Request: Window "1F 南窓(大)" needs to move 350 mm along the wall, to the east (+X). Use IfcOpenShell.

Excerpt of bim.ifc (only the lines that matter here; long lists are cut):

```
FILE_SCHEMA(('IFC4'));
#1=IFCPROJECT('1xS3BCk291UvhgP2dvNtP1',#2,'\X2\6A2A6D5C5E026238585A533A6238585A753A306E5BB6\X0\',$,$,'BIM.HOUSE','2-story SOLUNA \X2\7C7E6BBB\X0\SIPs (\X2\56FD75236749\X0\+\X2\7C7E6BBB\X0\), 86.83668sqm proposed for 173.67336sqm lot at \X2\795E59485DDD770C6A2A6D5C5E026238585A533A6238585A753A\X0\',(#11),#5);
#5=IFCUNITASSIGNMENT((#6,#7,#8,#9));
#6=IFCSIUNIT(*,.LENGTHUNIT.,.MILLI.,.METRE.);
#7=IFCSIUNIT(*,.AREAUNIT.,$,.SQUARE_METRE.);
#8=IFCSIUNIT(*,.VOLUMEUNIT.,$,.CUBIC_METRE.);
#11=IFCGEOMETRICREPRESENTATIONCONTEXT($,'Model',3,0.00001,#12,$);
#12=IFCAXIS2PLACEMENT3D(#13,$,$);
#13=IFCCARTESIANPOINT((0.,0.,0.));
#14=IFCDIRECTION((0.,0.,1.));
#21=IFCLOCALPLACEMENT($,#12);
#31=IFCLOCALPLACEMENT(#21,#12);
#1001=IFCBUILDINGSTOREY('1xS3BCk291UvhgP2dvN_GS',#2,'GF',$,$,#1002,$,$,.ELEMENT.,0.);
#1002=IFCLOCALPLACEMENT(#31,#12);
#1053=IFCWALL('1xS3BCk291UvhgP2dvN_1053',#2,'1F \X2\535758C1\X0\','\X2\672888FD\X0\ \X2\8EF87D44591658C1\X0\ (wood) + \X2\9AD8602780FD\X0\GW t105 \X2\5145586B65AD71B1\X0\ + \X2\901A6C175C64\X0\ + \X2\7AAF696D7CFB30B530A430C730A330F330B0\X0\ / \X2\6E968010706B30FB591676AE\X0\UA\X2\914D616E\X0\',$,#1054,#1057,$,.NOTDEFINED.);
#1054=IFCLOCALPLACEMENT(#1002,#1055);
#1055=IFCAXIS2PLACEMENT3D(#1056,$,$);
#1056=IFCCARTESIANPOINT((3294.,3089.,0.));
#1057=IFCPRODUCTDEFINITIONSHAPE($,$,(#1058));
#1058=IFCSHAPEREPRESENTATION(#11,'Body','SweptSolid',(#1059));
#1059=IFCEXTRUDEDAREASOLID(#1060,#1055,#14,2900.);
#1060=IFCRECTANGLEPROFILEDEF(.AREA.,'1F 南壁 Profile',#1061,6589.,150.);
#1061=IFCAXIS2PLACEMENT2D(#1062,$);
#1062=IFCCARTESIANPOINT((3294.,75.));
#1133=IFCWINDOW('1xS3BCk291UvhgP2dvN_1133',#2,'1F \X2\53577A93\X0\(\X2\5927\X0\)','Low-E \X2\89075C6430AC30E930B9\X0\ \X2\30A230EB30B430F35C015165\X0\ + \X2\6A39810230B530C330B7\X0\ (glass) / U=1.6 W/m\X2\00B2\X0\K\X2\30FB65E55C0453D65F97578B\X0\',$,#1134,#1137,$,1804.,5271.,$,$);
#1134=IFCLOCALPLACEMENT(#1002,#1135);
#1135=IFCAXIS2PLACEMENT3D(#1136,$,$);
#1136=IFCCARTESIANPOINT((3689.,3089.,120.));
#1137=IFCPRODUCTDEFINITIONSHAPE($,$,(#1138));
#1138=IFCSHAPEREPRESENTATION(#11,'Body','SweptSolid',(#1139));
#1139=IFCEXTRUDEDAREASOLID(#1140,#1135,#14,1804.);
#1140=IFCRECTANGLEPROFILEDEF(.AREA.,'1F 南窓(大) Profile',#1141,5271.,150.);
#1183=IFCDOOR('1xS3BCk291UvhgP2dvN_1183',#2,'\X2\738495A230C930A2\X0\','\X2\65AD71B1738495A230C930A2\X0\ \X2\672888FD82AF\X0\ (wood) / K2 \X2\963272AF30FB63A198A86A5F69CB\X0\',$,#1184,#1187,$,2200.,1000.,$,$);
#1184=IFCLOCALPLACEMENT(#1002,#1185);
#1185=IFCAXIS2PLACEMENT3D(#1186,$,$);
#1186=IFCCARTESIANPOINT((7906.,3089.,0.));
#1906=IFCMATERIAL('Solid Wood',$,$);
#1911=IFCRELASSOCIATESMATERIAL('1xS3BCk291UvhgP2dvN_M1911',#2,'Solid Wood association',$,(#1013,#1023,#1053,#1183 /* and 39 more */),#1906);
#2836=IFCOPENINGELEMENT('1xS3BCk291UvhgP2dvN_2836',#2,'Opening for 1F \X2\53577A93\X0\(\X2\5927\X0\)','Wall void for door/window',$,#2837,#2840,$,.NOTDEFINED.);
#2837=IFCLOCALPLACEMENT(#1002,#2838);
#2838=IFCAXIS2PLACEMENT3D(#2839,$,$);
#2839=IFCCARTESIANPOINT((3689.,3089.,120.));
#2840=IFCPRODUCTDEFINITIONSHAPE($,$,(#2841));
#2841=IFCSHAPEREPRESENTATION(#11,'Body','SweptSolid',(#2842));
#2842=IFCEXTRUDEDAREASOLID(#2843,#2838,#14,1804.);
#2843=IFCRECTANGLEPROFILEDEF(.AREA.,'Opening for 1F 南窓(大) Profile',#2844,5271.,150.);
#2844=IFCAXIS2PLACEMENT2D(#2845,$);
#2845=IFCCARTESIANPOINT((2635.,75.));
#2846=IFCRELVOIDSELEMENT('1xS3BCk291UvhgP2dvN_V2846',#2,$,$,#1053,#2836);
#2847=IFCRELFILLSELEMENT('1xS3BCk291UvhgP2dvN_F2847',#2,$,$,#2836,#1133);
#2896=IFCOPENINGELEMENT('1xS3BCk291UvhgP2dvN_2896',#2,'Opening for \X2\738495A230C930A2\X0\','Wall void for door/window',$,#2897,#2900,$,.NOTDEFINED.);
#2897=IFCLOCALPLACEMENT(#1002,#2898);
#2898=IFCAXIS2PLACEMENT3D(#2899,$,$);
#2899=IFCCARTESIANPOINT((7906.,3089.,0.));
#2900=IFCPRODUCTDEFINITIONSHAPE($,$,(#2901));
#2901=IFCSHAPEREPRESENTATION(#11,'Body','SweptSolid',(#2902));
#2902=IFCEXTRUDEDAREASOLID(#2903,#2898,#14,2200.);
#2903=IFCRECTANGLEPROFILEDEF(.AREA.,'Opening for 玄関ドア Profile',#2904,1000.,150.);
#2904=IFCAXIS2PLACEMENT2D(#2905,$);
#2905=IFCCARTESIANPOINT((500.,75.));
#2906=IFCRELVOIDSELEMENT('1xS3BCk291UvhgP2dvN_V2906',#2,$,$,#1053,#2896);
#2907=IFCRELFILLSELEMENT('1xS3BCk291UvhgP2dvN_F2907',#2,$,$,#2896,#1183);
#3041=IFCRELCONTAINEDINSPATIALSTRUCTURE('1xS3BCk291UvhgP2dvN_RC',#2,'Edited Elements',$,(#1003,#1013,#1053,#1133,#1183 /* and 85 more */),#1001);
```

```python
import ifcopenshell
import ifcopenshell.api.geometry
import ifcopenshell.util.placement
import ifcopenshell.util.unit

model = ifcopenshell.open("bim.ifc")
unit_scale = ifcopenshell.util.unit.calculate_unit_scale(model)

window = model.by_guid("1xS3BCk291UvhgP2dvN_1133")
opening = window.FillsVoids[0].RelatingOpeningElement
wall = opening.VoidsElements[0].RelatingBuildingElement

wall_matrix = ifcopenshell.util.placement.get_local_placement(wall.ObjectPlacement)
shift = wall_matrix[:3, 0] * 0.35 / unit_scale
before = ifcopenshell.util.placement.get_local_placement(window.ObjectPlacement)[:3, 3].copy()

# The window is not placed relative to its opening, so move both.
for product in (opening, window):
    matrix = ifcopenshell.util.placement.get_local_placement(product.ObjectPlacement)
    matrix[:3, 3] += shift
    ifcopenshell.api.geometry.edit_object_placement(model, product=product, matrix=matrix, is_si=False)

after = ifcopenshell.util.placement.get_local_placement(window.ObjectPlacement)[:3, 3]
print("window moved by", (after - before).round(3) + 0.0)

model.write("bim_rev.ifc")
```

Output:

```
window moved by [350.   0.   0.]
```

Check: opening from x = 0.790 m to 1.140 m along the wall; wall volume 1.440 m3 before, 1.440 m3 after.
